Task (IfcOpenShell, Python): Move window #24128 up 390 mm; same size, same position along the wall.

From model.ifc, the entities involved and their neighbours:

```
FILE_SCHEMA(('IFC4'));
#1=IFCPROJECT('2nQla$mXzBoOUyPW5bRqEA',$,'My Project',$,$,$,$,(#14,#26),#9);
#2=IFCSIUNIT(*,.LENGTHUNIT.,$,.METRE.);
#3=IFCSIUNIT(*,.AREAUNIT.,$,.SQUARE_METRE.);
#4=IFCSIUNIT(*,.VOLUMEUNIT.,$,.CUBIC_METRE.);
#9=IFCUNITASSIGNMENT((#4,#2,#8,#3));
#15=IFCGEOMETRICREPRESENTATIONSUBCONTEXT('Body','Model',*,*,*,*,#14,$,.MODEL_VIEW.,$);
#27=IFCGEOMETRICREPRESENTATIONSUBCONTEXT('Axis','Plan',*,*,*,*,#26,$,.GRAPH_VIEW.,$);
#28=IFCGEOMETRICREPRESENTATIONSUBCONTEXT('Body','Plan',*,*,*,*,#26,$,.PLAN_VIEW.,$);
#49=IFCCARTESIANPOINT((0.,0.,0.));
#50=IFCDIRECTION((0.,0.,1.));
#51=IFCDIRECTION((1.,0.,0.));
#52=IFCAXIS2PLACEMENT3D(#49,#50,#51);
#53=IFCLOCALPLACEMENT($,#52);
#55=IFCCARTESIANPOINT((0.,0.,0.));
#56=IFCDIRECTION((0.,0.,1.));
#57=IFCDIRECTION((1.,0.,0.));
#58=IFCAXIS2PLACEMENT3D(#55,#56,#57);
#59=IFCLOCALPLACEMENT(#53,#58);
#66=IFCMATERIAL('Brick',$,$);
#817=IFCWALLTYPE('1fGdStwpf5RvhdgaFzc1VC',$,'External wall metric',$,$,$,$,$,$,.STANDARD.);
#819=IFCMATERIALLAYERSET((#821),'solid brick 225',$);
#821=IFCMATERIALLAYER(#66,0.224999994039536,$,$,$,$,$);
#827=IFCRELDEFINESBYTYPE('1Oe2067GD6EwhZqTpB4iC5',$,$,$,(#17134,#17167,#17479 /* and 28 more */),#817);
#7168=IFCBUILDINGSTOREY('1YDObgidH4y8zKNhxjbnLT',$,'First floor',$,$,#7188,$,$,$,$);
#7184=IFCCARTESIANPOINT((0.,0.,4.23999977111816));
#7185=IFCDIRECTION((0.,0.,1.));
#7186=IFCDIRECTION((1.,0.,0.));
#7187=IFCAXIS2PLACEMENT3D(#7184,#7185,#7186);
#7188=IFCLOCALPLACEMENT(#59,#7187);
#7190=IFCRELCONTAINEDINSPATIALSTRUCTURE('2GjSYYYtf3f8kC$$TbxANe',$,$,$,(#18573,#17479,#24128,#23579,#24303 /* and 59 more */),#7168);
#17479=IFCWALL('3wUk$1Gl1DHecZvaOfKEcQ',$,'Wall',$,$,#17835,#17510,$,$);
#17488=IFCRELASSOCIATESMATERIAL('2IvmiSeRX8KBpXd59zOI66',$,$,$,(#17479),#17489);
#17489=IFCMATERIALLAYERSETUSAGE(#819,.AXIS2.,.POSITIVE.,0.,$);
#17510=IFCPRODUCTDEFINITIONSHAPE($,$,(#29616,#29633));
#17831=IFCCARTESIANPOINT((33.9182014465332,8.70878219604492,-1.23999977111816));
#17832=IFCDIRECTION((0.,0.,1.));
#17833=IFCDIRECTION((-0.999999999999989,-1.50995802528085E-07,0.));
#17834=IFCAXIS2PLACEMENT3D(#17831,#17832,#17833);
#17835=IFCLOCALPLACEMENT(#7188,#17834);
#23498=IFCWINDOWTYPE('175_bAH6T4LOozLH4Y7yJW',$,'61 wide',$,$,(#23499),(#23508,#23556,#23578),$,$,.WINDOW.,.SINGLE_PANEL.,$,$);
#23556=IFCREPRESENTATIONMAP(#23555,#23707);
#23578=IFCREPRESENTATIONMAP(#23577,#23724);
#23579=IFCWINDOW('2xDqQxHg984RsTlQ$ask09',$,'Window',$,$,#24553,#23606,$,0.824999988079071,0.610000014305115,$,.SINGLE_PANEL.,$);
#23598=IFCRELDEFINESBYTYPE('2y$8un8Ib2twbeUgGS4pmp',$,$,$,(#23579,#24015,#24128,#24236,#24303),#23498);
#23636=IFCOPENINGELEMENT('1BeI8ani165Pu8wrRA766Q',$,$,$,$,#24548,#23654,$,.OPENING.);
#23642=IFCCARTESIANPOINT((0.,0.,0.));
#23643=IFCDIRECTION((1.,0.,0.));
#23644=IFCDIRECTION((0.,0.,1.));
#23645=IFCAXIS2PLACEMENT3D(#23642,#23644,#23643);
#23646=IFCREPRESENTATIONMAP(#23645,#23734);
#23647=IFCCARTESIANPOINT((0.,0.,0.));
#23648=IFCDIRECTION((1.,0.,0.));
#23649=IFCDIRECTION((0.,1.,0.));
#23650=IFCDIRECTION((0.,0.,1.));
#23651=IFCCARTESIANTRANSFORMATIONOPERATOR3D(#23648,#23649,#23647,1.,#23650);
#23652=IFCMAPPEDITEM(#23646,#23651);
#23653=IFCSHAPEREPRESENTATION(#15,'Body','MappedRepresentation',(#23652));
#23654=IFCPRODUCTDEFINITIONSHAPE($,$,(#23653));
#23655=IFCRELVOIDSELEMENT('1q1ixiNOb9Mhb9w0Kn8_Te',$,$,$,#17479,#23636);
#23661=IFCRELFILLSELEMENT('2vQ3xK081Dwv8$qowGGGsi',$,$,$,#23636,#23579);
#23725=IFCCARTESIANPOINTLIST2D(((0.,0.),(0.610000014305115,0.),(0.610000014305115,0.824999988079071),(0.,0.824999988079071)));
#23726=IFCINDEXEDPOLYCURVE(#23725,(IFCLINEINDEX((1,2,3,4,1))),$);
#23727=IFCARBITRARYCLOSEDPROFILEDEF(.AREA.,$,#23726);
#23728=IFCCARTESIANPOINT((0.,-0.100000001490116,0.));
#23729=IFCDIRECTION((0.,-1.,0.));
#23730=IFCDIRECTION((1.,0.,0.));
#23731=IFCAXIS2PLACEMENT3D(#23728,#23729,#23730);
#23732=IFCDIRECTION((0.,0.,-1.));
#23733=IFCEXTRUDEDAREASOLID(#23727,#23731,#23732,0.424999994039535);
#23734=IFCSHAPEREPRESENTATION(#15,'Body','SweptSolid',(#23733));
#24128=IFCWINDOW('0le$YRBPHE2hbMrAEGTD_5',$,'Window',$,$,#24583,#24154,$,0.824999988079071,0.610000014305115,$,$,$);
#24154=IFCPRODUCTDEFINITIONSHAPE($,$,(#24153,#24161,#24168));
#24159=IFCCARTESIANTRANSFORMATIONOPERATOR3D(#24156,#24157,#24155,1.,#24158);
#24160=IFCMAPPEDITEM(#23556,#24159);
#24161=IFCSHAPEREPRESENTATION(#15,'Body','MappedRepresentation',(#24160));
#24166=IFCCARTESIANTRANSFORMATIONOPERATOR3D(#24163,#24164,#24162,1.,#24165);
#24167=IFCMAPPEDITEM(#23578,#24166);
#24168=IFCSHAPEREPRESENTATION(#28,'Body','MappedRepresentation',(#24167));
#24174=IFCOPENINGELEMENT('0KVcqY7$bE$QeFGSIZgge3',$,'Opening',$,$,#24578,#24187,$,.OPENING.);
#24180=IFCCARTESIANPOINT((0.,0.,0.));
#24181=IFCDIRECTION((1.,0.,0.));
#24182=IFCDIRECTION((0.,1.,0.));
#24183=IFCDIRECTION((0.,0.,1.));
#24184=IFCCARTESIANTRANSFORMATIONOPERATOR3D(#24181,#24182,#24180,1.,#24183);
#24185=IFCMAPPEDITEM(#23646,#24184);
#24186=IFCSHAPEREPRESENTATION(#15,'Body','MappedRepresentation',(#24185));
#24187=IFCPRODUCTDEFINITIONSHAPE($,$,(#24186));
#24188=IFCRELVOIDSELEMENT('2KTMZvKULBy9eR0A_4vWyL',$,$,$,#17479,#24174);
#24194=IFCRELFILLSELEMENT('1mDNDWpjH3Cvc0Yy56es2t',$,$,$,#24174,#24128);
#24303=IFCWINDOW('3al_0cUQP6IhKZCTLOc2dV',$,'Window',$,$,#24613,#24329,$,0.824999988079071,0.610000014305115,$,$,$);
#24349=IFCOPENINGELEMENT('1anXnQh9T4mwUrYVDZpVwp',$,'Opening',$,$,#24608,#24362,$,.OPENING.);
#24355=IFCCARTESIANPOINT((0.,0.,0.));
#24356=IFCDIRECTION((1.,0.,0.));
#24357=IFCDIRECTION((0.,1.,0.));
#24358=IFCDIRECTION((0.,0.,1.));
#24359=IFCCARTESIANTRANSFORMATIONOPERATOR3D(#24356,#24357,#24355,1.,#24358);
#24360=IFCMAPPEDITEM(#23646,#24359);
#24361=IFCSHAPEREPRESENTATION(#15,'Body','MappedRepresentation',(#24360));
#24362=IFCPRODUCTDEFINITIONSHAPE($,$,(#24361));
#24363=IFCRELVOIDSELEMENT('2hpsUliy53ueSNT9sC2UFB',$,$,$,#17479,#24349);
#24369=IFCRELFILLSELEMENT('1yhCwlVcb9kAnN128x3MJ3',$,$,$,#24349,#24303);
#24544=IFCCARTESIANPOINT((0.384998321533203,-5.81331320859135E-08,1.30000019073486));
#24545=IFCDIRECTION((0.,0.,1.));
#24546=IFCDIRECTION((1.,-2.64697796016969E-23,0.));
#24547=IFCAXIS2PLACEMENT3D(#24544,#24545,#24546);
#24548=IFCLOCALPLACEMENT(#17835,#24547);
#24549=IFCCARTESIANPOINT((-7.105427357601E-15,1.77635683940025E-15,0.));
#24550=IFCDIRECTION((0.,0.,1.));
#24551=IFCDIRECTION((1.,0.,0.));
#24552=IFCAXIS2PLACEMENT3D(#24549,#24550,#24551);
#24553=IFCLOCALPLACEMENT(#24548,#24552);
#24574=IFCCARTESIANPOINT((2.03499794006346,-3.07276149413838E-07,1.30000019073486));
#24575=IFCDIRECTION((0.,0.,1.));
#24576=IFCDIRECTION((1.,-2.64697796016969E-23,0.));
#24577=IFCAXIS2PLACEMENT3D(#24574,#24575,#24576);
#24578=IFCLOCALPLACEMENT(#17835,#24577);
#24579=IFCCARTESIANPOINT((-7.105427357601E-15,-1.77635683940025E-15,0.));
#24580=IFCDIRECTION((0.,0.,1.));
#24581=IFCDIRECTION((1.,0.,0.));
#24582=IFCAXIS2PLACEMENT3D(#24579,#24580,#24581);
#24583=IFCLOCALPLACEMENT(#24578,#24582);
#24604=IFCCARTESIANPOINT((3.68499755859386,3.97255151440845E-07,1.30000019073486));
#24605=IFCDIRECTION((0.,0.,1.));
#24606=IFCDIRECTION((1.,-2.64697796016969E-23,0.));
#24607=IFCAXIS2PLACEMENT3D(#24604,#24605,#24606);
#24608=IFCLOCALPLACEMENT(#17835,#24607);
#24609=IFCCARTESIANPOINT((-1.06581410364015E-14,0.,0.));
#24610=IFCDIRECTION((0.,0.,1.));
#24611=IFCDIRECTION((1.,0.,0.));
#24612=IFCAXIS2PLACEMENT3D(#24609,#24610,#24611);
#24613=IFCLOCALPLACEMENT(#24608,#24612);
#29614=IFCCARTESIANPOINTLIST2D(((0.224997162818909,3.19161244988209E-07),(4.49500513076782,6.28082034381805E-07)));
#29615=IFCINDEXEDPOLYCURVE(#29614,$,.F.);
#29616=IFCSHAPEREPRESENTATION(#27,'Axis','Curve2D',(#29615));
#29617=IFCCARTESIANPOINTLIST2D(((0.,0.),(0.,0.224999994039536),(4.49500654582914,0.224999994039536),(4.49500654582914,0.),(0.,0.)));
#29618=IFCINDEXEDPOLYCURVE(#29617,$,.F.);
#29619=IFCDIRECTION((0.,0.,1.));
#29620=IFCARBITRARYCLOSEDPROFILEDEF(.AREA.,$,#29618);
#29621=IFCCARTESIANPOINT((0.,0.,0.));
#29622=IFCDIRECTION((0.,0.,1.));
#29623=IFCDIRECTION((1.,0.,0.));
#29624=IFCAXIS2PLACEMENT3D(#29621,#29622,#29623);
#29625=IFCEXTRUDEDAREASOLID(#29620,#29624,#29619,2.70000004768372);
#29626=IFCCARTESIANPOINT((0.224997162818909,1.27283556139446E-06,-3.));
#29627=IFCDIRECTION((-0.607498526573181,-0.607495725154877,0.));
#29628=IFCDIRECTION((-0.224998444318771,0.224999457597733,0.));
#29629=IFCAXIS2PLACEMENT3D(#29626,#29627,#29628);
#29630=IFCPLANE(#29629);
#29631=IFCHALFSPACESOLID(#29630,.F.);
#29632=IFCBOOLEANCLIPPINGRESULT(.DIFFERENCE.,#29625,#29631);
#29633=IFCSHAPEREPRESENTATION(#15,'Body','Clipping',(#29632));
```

```python
import numpy as np
import ifcopenshell
import ifcopenshell.api.geometry
import ifcopenshell.util.placement
import ifcopenshell.util.unit

model = ifcopenshell.open("model.ifc")
unit_scale = ifcopenshell.util.unit.calculate_unit_scale(model)

window = model.by_guid("0le$YRBPHE2hbMrAEGTD_5")
opening = window.FillsVoids[0].RelatingOpeningElement
dz = 0.39 / unit_scale

shift = np.array([0.0, 0.0, dz])
# The window is placed relative to its opening, so it follows when the opening moves.
matrix = ifcopenshell.util.placement.get_local_placement(opening.ObjectPlacement)
matrix[:3, 3] += shift
ifcopenshell.api.geometry.edit_object_placement(
    model, product=opening, matrix=matrix, is_si=False, should_transform_children=True
)

print(f"moved by {dz * unit_scale:+.3f} m")

model.write("model-out.ifc")
```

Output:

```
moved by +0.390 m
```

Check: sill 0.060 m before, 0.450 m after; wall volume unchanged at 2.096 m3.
